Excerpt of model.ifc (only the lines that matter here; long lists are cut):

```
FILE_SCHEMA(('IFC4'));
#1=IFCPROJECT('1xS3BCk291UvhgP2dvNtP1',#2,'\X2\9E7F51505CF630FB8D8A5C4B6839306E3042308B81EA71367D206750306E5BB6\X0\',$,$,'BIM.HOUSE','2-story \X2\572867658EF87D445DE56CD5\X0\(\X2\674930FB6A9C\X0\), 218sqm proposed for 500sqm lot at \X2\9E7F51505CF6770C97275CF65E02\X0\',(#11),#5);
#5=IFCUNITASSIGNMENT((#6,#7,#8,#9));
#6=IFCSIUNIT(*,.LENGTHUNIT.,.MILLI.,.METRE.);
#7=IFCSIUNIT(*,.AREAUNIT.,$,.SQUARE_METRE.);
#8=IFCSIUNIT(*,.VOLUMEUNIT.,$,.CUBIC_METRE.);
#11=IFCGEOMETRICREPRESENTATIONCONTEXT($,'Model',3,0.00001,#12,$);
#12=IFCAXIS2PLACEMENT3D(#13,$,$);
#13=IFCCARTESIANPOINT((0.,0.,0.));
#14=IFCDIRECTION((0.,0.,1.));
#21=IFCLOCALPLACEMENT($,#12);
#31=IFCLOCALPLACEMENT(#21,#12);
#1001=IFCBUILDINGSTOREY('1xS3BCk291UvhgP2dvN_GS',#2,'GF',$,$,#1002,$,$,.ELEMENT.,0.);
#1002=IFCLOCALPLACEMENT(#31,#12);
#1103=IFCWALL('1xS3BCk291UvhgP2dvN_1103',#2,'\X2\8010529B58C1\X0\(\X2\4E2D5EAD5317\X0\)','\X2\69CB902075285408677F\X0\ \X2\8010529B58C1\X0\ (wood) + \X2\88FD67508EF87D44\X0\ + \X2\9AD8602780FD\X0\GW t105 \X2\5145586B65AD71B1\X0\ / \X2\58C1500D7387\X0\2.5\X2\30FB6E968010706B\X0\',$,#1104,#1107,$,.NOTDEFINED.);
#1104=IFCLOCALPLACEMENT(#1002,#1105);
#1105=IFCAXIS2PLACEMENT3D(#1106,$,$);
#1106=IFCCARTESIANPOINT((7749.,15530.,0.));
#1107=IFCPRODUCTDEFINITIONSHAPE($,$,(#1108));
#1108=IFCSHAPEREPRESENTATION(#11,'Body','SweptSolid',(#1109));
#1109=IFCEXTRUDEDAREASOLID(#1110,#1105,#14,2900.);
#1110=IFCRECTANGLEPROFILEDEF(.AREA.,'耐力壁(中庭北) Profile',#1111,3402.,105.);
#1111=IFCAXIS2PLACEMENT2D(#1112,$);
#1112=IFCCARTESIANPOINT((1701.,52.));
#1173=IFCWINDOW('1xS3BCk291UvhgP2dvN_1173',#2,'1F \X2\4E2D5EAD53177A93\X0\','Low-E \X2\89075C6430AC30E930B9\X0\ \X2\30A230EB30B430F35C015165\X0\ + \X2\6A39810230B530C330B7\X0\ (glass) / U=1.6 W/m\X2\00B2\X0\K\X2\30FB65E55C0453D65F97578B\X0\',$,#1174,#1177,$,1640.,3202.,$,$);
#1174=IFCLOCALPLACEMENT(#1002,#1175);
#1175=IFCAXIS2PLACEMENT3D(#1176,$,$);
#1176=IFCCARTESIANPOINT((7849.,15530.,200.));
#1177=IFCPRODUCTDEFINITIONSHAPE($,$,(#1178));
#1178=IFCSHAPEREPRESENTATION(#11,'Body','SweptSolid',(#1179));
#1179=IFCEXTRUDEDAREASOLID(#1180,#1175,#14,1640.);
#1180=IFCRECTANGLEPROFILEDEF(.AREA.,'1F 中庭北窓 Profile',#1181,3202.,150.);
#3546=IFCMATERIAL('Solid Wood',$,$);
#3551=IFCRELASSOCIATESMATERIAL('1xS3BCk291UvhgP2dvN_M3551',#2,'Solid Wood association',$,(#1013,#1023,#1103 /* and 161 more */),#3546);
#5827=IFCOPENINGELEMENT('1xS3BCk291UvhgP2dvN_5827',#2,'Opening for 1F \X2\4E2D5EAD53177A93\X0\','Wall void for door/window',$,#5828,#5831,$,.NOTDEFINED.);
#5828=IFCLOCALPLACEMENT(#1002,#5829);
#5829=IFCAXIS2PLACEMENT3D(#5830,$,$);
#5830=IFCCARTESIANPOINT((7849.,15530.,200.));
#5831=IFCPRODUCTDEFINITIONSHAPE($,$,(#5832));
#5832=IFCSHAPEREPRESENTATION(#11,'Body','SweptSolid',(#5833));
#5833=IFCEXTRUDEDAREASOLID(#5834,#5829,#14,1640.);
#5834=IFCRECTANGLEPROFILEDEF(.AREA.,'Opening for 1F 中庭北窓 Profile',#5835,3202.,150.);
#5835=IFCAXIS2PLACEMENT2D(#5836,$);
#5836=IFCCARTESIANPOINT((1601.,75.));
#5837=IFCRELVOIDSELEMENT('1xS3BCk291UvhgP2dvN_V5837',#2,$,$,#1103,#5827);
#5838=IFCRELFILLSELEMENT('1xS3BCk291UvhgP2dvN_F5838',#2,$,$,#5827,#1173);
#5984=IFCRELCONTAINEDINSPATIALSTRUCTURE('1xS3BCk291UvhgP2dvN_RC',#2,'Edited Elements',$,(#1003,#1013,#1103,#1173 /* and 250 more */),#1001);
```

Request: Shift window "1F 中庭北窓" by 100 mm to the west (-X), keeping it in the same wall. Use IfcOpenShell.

```python
import ifcopenshell
import ifcopenshell.api.geometry
import ifcopenshell.util.placement
import ifcopenshell.util.unit

model = ifcopenshell.open("model.ifc")
unit_scale = ifcopenshell.util.unit.calculate_unit_scale(model)

window = model.by_guid("1xS3BCk291UvhgP2dvN_1173")
opening = window.FillsVoids[0].RelatingOpeningElement
wall = opening.VoidsElements[0].RelatingBuildingElement

wall_matrix = ifcopenshell.util.placement.get_local_placement(wall.ObjectPlacement)
shift = wall_matrix[:3, 0] * -0.1 / unit_scale
before = ifcopenshell.util.placement.get_local_placement(window.ObjectPlacement)[:3, 3].copy()

# The window is not placed relative to its opening, so move both.
for product in (opening, window):
    matrix = ifcopenshell.util.placement.get_local_placement(product.ObjectPlacement)
    matrix[:3, 3] += shift
    ifcopenshell.api.geometry.edit_object_placement(model, product=product, matrix=matrix, is_si=False)

after = ifcopenshell.util.placement.get_local_placement(window.ObjectPlacement)[:3, 3]
print("window moved by", (after - before).round(3) + 0.0)

model.write("model_updated.ifc")
```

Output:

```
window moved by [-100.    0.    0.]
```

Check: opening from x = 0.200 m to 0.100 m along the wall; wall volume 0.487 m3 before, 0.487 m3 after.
